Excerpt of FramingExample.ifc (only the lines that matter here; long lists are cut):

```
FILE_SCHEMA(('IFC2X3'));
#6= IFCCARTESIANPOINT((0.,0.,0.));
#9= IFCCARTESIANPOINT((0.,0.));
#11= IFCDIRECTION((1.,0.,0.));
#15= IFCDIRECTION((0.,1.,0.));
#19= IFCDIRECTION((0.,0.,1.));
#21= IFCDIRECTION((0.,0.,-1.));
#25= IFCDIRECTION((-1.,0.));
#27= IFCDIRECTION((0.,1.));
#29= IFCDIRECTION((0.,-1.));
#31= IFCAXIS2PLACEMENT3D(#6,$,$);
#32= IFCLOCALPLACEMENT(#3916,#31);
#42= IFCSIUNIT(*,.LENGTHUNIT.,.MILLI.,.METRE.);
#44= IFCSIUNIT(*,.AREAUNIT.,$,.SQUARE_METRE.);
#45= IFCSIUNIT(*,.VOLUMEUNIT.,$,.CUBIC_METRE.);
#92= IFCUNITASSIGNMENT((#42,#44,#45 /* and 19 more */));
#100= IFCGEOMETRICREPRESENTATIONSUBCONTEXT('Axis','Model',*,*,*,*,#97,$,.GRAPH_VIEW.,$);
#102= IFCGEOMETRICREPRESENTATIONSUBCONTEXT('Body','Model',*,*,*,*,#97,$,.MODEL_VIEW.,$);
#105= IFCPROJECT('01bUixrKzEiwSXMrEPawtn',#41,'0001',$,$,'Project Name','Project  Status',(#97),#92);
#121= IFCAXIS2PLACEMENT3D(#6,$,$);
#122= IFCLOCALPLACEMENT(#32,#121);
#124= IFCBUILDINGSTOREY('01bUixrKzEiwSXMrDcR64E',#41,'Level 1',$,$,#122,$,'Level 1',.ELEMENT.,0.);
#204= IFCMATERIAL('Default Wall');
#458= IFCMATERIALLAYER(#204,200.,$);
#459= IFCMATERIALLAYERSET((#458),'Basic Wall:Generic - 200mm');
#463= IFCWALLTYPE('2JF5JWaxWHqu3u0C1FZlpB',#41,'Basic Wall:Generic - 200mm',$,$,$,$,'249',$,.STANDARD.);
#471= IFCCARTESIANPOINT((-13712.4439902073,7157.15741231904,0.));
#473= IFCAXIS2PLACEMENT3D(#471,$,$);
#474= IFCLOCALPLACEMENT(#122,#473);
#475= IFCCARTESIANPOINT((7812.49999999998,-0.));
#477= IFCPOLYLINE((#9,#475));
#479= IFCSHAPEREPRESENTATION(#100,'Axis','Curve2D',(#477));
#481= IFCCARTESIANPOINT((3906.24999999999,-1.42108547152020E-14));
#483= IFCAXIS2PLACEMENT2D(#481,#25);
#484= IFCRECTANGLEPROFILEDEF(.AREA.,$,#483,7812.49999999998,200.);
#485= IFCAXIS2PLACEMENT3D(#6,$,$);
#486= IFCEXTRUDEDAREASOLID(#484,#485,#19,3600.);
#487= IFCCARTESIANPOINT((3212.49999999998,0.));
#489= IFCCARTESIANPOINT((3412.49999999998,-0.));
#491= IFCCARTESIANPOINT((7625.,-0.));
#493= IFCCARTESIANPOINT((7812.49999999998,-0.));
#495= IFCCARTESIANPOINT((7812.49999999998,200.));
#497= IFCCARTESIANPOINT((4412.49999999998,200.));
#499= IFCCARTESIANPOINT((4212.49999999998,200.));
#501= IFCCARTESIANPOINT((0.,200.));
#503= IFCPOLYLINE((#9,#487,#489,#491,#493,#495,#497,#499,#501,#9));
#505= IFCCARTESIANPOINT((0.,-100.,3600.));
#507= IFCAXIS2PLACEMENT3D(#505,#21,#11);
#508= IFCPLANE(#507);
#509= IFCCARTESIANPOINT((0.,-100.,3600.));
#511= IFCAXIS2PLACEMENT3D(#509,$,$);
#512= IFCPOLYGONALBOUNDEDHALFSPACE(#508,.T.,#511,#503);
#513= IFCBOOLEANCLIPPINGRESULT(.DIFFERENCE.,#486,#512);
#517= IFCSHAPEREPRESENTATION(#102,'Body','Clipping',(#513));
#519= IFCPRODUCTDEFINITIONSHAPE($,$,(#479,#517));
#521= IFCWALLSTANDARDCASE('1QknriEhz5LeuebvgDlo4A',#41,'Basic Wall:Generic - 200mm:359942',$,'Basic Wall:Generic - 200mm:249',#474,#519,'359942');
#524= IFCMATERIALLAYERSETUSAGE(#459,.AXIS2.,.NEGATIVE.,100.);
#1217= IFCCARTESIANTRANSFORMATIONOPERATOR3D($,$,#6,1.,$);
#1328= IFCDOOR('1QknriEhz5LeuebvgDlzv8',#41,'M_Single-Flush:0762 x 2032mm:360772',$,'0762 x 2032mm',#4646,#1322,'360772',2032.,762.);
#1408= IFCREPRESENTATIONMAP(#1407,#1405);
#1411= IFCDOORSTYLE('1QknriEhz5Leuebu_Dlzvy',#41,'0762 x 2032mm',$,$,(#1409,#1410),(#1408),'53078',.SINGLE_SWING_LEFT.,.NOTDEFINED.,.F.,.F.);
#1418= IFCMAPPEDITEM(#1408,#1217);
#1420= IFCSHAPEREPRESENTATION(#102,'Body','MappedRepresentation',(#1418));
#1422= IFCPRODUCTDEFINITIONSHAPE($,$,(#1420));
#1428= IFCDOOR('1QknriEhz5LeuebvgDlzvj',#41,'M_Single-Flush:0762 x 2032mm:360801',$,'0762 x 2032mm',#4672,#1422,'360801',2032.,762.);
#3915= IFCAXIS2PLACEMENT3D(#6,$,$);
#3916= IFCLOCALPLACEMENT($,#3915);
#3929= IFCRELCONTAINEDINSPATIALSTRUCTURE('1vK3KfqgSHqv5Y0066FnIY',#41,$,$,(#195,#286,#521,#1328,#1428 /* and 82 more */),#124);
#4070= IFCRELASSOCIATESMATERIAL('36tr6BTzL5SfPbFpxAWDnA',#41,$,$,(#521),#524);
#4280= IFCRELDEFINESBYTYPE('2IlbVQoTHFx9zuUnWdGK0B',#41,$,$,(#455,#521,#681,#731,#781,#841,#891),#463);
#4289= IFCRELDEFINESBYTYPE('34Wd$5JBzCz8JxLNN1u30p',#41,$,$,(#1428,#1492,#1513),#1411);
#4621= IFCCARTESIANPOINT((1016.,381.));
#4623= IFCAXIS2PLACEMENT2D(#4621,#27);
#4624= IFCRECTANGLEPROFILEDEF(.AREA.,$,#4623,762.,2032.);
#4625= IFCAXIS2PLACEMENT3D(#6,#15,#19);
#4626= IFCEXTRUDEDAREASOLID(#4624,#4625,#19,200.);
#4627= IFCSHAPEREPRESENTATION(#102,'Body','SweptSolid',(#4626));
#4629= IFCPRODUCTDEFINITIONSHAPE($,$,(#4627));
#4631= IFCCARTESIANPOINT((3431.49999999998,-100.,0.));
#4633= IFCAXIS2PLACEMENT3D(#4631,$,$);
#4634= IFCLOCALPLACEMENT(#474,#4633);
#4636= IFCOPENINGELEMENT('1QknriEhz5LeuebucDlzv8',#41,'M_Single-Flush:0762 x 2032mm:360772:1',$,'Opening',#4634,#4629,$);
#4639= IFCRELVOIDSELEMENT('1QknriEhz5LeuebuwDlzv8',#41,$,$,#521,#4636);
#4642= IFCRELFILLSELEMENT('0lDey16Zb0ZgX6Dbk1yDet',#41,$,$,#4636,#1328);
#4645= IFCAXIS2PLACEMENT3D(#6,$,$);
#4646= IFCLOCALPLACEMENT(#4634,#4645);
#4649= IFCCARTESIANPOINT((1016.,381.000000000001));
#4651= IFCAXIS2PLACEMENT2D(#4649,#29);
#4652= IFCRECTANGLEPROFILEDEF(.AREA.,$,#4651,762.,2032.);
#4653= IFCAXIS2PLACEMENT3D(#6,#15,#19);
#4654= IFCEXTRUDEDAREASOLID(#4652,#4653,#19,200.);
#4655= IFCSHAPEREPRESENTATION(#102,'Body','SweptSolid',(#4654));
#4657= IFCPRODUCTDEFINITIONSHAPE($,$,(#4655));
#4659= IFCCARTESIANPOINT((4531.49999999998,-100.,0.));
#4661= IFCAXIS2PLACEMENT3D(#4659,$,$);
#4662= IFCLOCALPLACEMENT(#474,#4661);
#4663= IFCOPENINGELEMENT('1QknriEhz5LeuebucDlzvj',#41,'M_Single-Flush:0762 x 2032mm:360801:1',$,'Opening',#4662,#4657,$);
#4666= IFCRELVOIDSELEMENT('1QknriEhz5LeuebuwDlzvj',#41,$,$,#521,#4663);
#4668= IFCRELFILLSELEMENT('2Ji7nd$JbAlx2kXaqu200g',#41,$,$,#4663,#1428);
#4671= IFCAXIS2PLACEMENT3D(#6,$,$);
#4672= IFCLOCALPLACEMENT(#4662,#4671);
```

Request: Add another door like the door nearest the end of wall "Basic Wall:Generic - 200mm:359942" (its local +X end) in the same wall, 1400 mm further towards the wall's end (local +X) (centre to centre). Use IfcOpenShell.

```python
import ifcopenshell
import ifcopenshell.api.feature
import ifcopenshell.api.geometry
import ifcopenshell.api.root
import ifcopenshell.geom
import ifcopenshell.util.element
import ifcopenshell.util.placement
import ifcopenshell.util.shape

model = ifcopenshell.open("FramingExample.ifc")
settings = ifcopenshell.geom.settings()


def volume(element):
    """Net volume in cubic metres, openings subtracted."""
    shape = ifcopenshell.geom.create_shape(settings, element)
    return ifcopenshell.util.shape.get_volume(shape.geometry)


def reuse_history(source, copy):
    """copy_class also copies each property set's owner history, people and application; keep the originals."""
    for rel in copy.IsDefinedBy:
        if rel.is_a("IfcRelDefinesByProperties") and (history := rel.RelatingPropertyDefinition.OwnerHistory):
            rel.RelatingPropertyDefinition.OwnerHistory = source.OwnerHistory
            ifcopenshell.util.element.remove_deep2(model, history)


door = model.by_guid("1QknriEhz5LeuebvgDlzvj")
opening = door.FillsVoids[0].RelatingOpeningElement
wall = opening.VoidsElements[0].RelatingBuildingElement
before = volume(wall)
shift = ifcopenshell.util.placement.get_local_placement(wall.ObjectPlacement)[:3, 0] * 1400.0

# copy_class copies the void relationship, type, container and properties, but no geometry.
new_opening = ifcopenshell.api.root.copy_class(model, product=opening)
new_opening.Representation = ifcopenshell.util.element.copy_deep(
    model, opening.Representation, exclude=["IfcGeometricRepresentationContext", "IfcRepresentationMap"]
)
new_opening.Name = "M_Single-Flush:0762 x 2032mm"
new_door = ifcopenshell.api.root.copy_class(model, product=door)
new_door.Representation = ifcopenshell.util.element.copy_deep(
    model, door.Representation, exclude=["IfcGeometricRepresentationContext", "IfcRepresentationMap"]
)
new_door.Name = "M_Single-Flush:0762 x 2032mm"
new_door.Tag = None
reuse_history(door, new_door)
fills = ifcopenshell.api.feature.add_filling(model, opening=new_opening, element=new_door)
fills.OwnerHistory = new_door.OwnerHistory  # required in IFC2X3

for old, new in ((opening, new_opening), (door, new_door)):
    matrix = ifcopenshell.util.placement.get_local_placement(old.ObjectPlacement)
    matrix[:3, 3] += shift
    ifcopenshell.api.geometry.edit_object_placement(model, product=new, matrix=matrix, is_si=False)

after = volume(wall)

print(f"wall volume {before:.3f} -> {after:.3f} m3")

model.write("FramingExample_v2.ifc")
```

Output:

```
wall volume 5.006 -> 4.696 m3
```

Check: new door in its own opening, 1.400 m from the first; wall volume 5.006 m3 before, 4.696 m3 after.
